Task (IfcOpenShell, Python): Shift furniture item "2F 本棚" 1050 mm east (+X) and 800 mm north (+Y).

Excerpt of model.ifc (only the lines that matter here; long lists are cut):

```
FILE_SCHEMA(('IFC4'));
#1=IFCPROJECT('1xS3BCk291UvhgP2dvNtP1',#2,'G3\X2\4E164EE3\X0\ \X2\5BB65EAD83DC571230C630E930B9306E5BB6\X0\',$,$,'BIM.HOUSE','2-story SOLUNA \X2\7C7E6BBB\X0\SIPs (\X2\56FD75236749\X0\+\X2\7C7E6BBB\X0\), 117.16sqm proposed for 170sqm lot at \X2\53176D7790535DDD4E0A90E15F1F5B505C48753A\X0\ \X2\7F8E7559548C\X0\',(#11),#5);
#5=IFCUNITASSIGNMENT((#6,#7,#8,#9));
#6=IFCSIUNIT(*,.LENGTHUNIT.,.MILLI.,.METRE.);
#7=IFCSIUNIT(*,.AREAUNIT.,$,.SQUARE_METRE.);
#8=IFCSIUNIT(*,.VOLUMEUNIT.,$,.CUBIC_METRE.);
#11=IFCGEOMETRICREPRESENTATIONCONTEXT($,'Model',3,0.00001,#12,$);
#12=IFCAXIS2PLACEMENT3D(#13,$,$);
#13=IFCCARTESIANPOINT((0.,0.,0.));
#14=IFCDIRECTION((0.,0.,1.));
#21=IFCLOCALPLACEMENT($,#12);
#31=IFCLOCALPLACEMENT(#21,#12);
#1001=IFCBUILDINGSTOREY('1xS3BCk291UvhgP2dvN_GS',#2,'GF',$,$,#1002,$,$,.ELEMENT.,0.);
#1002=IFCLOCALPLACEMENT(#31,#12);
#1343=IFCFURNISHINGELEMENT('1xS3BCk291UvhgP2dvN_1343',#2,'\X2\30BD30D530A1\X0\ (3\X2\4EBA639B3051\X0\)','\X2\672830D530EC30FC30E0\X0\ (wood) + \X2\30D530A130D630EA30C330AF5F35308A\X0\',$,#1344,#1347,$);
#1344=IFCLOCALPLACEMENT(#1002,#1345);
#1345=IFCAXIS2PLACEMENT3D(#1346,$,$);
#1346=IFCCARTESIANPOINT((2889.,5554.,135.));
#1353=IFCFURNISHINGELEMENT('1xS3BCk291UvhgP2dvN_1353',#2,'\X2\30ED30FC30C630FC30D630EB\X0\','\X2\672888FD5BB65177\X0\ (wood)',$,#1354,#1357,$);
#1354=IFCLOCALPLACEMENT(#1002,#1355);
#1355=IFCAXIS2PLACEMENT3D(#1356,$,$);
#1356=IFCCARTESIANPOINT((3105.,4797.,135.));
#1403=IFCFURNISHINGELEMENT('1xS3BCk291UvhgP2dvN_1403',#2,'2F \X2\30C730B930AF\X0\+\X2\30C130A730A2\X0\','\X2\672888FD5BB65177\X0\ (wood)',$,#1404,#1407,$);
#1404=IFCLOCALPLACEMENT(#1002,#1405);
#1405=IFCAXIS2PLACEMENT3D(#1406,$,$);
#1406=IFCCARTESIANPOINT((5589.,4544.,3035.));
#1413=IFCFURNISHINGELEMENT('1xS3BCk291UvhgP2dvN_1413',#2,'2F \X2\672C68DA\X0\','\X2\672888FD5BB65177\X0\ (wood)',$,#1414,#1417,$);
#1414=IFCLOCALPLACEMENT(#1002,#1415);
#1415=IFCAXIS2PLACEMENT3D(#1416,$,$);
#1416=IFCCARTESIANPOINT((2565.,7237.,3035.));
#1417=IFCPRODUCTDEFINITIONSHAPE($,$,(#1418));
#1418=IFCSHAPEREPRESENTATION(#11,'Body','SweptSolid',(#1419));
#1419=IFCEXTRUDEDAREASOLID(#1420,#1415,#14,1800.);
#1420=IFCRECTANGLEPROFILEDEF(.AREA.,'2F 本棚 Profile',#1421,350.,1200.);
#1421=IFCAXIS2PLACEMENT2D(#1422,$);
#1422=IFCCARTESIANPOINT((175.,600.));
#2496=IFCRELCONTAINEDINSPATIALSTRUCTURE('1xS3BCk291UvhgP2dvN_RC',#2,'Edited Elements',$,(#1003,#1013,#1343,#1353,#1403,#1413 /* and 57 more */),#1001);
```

```python
import ifcopenshell
import ifcopenshell.api.geometry
import ifcopenshell.util.placement
import ifcopenshell.util.unit

model = ifcopenshell.open("model.ifc")
unit_scale = ifcopenshell.util.unit.calculate_unit_scale(model)

item = model.by_guid("1xS3BCk291UvhgP2dvN_1413")
matrix = ifcopenshell.util.placement.get_local_placement(item.ObjectPlacement)
matrix[0, 3] += 1.05 / unit_scale
matrix[1, 3] += 0.8 / unit_scale
ifcopenshell.api.geometry.edit_object_placement(model, product=item, matrix=matrix, is_si=False)

print(ifcopenshell.util.placement.get_local_placement(item.ObjectPlacement).round(3) + 0.0)

model.write("model_rev.ifc")
```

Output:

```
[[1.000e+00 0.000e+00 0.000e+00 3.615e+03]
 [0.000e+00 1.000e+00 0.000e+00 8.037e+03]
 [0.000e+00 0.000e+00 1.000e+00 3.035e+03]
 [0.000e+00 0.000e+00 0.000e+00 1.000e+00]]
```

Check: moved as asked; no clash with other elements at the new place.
